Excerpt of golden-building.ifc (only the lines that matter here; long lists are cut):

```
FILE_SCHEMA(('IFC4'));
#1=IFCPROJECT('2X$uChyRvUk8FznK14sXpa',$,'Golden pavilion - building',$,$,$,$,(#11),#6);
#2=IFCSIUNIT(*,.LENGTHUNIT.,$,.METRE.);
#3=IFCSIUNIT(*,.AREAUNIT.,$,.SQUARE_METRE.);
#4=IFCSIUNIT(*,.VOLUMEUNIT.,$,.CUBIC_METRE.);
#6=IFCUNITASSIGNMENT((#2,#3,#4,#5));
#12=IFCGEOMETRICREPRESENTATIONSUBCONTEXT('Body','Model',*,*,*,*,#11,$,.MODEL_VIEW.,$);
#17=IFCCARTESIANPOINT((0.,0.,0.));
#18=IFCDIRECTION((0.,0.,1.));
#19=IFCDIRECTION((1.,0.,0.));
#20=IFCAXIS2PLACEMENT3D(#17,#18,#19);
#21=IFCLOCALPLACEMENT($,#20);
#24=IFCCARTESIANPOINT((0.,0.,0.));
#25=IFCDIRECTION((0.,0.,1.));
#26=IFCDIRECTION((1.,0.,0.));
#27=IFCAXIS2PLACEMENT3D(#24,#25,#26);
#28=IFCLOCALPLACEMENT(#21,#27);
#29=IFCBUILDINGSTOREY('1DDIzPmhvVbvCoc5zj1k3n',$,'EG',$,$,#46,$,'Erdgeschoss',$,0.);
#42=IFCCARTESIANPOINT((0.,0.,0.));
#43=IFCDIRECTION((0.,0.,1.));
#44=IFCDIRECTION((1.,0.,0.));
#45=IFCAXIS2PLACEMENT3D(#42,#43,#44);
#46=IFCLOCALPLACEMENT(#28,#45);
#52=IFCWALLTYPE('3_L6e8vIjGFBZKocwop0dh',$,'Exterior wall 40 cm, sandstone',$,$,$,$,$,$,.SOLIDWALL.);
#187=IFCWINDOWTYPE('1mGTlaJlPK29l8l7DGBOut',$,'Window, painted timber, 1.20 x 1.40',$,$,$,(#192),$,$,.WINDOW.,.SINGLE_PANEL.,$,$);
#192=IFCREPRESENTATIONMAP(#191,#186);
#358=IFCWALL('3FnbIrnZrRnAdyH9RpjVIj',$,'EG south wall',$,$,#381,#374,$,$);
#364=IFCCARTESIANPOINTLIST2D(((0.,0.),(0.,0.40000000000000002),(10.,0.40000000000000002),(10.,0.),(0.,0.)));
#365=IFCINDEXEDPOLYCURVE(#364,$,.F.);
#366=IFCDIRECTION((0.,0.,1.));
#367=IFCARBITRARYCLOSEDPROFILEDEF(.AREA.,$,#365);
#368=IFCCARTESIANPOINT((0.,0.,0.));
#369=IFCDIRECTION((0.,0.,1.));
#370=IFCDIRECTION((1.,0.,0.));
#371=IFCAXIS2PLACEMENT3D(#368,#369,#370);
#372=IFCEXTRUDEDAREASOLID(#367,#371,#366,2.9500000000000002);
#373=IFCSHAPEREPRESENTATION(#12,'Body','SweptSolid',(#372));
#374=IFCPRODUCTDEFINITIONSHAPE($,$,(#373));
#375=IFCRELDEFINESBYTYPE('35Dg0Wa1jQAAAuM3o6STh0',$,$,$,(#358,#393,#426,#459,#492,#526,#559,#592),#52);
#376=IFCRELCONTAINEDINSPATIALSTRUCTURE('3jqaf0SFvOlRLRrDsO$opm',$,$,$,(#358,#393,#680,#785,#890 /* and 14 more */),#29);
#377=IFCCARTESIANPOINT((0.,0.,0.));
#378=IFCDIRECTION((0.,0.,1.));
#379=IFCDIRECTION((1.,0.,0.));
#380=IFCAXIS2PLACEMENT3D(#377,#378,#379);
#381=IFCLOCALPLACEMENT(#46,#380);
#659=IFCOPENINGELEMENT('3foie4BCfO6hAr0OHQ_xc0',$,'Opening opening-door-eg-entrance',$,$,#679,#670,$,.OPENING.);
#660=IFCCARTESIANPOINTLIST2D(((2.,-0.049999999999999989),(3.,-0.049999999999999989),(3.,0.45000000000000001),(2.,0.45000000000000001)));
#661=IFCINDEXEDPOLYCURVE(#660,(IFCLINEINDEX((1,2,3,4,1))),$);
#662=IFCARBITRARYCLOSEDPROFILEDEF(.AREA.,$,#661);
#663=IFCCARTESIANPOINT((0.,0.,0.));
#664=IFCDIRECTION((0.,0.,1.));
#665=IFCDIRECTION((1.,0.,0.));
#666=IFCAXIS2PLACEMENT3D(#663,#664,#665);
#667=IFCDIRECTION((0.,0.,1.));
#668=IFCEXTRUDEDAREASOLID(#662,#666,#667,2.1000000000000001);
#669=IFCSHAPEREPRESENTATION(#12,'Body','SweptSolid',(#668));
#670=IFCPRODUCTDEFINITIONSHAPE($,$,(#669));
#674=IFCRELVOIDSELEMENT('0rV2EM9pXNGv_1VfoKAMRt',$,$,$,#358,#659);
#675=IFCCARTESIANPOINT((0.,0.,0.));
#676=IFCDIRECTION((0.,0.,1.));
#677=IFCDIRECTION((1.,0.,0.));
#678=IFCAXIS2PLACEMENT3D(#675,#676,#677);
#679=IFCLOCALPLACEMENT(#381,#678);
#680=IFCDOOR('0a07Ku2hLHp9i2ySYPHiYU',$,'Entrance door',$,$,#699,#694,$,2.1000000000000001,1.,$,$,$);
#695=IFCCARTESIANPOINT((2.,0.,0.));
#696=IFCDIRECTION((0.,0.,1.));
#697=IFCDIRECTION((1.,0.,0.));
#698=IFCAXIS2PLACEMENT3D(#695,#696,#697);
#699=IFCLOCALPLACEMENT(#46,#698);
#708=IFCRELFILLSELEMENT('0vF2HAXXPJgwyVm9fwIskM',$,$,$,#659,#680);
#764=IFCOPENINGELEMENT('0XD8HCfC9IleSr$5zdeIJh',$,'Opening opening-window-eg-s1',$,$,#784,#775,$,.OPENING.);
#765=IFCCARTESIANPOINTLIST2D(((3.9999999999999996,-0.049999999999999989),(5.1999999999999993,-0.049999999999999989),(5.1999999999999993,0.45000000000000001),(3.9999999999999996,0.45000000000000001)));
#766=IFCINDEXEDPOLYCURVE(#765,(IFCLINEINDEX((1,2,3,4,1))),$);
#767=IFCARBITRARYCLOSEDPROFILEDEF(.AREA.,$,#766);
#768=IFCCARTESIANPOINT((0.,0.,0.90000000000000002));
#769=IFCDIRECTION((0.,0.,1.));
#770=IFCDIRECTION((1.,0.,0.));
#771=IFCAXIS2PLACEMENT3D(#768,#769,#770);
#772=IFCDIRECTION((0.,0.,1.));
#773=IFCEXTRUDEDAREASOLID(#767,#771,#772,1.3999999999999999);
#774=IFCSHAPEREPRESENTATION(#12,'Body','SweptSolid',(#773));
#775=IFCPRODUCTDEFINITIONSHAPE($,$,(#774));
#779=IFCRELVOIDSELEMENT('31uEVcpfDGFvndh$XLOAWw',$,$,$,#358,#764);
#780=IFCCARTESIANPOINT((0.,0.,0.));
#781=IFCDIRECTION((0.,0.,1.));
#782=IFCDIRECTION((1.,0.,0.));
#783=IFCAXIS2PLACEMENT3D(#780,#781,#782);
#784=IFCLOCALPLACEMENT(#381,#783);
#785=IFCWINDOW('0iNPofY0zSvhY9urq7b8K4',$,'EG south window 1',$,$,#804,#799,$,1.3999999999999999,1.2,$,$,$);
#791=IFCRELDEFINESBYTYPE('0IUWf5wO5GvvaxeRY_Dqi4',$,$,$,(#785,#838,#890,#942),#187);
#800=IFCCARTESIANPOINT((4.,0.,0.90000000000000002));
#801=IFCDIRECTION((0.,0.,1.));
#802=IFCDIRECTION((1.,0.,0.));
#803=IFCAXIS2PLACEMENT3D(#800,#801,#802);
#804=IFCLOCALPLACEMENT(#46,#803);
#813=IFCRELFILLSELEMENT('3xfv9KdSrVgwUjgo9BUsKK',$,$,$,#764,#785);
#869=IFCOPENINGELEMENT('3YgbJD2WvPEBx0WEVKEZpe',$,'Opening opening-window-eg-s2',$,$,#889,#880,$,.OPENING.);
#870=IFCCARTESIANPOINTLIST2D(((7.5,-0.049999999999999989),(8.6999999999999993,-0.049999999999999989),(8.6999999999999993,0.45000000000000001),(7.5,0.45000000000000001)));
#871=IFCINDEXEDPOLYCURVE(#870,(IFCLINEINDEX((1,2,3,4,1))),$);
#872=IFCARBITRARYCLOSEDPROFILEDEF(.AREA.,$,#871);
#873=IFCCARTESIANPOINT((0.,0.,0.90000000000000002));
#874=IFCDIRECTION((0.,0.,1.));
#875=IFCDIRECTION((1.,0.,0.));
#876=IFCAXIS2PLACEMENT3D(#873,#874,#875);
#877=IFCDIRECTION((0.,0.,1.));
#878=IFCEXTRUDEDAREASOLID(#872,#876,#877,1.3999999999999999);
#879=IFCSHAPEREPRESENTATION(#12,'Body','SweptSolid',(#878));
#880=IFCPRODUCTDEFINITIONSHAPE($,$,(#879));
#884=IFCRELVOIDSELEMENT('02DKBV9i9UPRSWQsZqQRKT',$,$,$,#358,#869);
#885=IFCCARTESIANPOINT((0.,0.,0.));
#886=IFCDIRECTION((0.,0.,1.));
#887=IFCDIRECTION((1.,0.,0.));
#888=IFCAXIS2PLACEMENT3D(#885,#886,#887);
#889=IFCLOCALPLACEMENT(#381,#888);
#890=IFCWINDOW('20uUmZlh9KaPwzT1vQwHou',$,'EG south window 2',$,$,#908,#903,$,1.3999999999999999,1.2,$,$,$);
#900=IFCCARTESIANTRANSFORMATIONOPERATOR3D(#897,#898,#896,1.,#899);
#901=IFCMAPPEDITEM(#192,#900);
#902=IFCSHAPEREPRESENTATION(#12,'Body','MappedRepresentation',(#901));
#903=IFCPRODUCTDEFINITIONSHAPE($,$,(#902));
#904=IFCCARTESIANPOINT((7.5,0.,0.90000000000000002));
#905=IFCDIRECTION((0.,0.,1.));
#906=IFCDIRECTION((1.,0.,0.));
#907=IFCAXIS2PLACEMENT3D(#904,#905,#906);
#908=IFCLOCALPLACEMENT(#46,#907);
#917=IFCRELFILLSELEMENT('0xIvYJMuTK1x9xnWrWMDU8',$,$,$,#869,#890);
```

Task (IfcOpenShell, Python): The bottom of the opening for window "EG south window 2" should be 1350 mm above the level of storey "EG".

```python
import numpy as np
import ifcopenshell
import ifcopenshell.api.geometry
import ifcopenshell.geom
import ifcopenshell.util.element
import ifcopenshell.util.placement
import ifcopenshell.util.shape
import ifcopenshell.util.unit

model = ifcopenshell.open("golden-building.ifc")
unit_scale = ifcopenshell.util.unit.calculate_unit_scale(model)

window = model.by_guid("20uUmZlh9KaPwzT1vQwHou")
opening = window.FillsVoids[0].RelatingOpeningElement
storey = ifcopenshell.util.element.get_container(window, ifc_class="IfcBuildingStorey")
level = ifcopenshell.util.placement.get_local_placement(storey.ObjectPlacement)[2, 3]

# The opening's origin need not be at the sill, so measure its lowest point.
shape = ifcopenshell.geom.create_shape(ifcopenshell.geom.settings(), opening)
bottom = ifcopenshell.util.shape.get_shape_bottom_elevation(shape, shape.geometry) / unit_scale
dz = level + 1.35 - bottom

shift = np.array([0.0, 0.0, dz])
# The window is not placed relative to its opening, so move both.
for product in (opening, window):
    matrix = ifcopenshell.util.placement.get_local_placement(product.ObjectPlacement)
    matrix[:3, 3] += shift
    ifcopenshell.api.geometry.edit_object_placement(model, product=product, matrix=matrix, is_si=False)

print(f"moved by {dz * unit_scale:+.3f} m")

model.write("golden-building_v2.ifc")
```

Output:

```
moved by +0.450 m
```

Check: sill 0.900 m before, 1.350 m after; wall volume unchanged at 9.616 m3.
